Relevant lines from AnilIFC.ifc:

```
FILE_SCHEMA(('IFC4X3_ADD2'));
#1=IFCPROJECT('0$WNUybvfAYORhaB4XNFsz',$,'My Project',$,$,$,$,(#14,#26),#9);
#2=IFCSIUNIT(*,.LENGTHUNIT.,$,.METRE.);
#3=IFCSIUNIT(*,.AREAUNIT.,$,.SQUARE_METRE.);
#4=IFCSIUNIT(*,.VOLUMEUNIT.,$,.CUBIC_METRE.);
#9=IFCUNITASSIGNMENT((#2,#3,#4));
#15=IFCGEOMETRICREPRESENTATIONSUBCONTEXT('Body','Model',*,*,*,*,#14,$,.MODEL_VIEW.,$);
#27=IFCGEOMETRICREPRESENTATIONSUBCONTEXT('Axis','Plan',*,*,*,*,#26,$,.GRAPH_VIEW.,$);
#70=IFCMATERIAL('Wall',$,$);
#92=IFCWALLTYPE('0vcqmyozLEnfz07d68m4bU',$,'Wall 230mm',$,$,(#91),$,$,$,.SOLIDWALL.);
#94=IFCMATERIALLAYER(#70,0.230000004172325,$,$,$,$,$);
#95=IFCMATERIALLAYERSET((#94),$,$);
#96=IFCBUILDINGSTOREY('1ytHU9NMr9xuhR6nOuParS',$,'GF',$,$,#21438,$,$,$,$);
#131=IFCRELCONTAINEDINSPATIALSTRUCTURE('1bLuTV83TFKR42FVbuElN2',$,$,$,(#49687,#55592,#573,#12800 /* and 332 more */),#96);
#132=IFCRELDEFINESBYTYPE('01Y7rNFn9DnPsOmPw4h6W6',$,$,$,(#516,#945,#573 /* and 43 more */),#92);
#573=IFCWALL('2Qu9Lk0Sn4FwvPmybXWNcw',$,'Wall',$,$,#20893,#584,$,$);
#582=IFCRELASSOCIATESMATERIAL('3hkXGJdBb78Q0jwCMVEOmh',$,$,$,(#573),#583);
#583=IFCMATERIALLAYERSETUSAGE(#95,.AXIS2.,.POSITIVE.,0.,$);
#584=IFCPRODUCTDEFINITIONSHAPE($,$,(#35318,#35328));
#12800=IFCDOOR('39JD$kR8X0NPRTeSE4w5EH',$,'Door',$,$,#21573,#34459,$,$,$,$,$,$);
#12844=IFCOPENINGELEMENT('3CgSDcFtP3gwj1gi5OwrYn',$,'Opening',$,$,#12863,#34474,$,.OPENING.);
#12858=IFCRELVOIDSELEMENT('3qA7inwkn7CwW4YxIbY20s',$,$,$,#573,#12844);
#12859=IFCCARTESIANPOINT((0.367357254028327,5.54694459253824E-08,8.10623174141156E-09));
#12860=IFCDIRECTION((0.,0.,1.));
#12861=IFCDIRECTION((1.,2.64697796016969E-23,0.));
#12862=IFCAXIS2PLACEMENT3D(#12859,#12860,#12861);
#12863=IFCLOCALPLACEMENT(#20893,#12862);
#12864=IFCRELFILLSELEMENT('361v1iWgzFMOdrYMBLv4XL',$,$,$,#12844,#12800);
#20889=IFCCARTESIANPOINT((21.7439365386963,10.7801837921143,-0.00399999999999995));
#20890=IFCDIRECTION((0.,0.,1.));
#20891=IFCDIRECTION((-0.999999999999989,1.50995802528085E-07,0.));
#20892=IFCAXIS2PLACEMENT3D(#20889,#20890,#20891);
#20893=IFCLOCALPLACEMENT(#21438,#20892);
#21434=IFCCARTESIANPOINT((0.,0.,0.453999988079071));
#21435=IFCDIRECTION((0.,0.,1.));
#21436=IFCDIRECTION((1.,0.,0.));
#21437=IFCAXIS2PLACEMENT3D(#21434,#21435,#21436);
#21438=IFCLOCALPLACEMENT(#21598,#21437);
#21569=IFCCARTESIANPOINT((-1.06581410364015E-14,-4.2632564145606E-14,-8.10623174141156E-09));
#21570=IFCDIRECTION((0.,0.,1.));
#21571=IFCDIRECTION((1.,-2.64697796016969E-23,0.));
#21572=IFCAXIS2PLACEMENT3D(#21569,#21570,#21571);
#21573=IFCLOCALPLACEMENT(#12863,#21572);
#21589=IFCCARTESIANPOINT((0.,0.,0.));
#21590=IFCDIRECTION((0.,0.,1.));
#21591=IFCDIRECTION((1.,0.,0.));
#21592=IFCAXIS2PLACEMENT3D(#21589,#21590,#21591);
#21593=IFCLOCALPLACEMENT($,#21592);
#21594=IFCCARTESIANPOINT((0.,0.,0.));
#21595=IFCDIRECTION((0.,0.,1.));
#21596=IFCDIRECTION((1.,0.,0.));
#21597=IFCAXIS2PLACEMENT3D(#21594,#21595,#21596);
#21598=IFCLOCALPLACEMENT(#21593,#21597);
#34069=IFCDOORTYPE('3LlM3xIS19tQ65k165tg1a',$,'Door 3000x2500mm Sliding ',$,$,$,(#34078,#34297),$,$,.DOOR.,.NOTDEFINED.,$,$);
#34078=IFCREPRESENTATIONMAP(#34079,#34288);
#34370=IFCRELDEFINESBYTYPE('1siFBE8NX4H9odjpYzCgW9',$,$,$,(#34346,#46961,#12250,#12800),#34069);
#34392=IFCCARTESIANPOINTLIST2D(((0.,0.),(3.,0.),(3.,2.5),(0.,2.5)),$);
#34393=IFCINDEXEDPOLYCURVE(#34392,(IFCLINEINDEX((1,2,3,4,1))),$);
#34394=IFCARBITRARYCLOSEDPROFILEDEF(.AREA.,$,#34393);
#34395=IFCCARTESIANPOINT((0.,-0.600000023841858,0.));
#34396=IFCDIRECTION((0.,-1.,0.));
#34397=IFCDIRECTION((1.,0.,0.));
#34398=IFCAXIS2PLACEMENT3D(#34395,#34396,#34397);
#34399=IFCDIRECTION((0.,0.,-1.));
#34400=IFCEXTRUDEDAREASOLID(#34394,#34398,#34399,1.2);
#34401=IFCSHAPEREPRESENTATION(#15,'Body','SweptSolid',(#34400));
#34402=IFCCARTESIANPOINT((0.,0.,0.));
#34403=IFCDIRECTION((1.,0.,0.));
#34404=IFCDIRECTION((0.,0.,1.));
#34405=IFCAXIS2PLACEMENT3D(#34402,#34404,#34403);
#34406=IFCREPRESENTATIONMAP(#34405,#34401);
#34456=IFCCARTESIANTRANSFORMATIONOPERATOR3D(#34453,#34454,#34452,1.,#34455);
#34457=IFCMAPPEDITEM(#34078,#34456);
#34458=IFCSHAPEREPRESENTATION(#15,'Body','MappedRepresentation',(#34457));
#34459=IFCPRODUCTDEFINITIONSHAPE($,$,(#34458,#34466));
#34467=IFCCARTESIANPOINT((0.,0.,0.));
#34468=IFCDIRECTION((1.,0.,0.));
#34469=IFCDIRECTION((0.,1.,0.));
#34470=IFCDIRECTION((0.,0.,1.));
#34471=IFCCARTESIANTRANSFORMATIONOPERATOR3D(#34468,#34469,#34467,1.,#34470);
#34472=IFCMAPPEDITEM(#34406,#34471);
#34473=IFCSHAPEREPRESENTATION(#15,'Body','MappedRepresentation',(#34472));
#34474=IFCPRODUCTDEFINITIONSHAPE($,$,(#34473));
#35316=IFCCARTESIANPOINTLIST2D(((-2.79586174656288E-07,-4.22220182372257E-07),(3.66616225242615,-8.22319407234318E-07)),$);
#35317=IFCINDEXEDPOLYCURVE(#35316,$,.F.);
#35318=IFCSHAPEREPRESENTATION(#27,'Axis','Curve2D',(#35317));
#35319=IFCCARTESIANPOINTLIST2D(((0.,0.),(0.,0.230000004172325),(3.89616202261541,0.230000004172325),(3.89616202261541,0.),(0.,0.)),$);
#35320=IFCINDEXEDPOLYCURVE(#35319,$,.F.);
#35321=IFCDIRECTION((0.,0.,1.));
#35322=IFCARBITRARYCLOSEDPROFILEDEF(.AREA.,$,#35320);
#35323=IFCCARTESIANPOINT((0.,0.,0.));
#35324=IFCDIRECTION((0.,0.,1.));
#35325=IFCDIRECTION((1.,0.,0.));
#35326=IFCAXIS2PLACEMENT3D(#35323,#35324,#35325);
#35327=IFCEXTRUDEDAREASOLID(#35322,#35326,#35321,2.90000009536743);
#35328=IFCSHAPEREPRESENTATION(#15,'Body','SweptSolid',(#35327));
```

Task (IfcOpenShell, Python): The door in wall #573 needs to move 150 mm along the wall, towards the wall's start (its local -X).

```python
import ifcopenshell
import ifcopenshell.api.geometry
import ifcopenshell.util.placement
import ifcopenshell.util.unit

model = ifcopenshell.open("AnilIFC.ifc")
unit_scale = ifcopenshell.util.unit.calculate_unit_scale(model)

door = model.by_guid("39JD$kR8X0NPRTeSE4w5EH")
opening = door.FillsVoids[0].RelatingOpeningElement
wall = opening.VoidsElements[0].RelatingBuildingElement

wall_matrix = ifcopenshell.util.placement.get_local_placement(wall.ObjectPlacement)
shift = wall_matrix[:3, 0] * -0.15 / unit_scale
before = ifcopenshell.util.placement.get_local_placement(door.ObjectPlacement)[:3, 3].copy()

# The door is placed relative to its opening, so it follows when the opening moves.
matrix = ifcopenshell.util.placement.get_local_placement(opening.ObjectPlacement)
matrix[:3, 3] += shift
ifcopenshell.api.geometry.edit_object_placement(
    model, product=opening, matrix=matrix, is_si=False, should_transform_children=True
)

after = ifcopenshell.util.placement.get_local_placement(door.ObjectPlacement)[:3, 3]
print("door moved by", (after - before).round(3) + 0.0)

model.write("AnilIFC_updated.ifc")
```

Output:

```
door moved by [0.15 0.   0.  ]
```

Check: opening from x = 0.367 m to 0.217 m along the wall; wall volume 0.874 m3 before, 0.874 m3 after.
